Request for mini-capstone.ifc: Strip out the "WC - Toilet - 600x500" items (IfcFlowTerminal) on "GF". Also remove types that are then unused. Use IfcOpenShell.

First a look at what the model holds.

```python
import ifcopenshell
import ifcopenshell.util.element

model = ifcopenshell.open("mini-capstone.ifc")
print(model.schema)
storey = next(s for s in model.by_type("IfcBuildingStorey") if s.Name == "GF")
terminals = [e for e in ifcopenshell.util.element.get_decomposition(storey) if e.is_a("IfcFlowTerminal")]
seen = {}
for e in terminals:
    element_type = ifcopenshell.util.element.get_type(e)
    name = element_type.Name if element_type not in (None, e) else None
    seen[name] = seen.get(name, 0) + 1
for name, count in sorted(seen.items(), key=str):
    print(count, "x", name)
```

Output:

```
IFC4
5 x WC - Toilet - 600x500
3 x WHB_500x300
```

```python
import ifcopenshell
import ifcopenshell.api.root
import ifcopenshell.util.element

model = ifcopenshell.open("mini-capstone.ifc")

storey = next(s for s in model.by_type("IfcBuildingStorey") if s.Name == "GF")
terminals = [e for e in ifcopenshell.util.element.get_decomposition(storey) if e.is_a("IfcFlowTerminal")]
targets = [e for e in terminals if (t := ifcopenshell.util.element.get_type(e)) not in (None, e) and t.Name == "WC - Toilet - 600x500"]
types = {ifcopenshell.util.element.get_type(e) for e in targets} - {None, *targets}

for e in targets:
    ifcopenshell.api.root.remove_product(model, product=e)
print(len(targets), "removed")

unused = [t for t in types if not ifcopenshell.util.element.get_types(t)]
for t in unused:
    ifcopenshell.api.root.remove_product(model, product=t)
print(len(unused), "unused types removed")

model.write("mini-capstone_v2.ifc")
```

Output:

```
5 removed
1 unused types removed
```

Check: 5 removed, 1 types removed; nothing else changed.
